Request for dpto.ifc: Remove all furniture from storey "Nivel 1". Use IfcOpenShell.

First a look at what the model holds.

```python
import ifcopenshell
import ifcopenshell.util.element

model = ifcopenshell.open("dpto.ifc")
print(model.schema)
storey = next(s for s in model.by_type("IfcBuildingStorey") if s.Name == "Nivel 1")
furniture = [e for e in ifcopenshell.util.element.get_decomposition(storey) if e.is_a("IfcFurnishingElement")]
seen = {}
for e in furniture:
    element_type = ifcopenshell.util.element.get_type(e)
    name = element_type.Name if element_type not in (None, e) else None
    seen[name] = seen.get(name, 0) + 1
for name, count in sorted(seen.items(), key=str):
    print(count, "x", name)
```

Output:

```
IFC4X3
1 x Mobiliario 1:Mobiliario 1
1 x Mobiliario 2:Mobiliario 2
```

```python
import ifcopenshell
import ifcopenshell.api.root
import ifcopenshell.util.element

model = ifcopenshell.open("dpto.ifc")

storey = next(s for s in model.by_type("IfcBuildingStorey") if s.Name == "Nivel 1")
furniture = [e for e in ifcopenshell.util.element.get_decomposition(storey) if e.is_a("IfcFurnishingElement")]

for e in furniture:
    ifcopenshell.api.root.remove_product(model, product=e)
print(len(furniture), "removed")

model.write("dpto_edited.ifc")
```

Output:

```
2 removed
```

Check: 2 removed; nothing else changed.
